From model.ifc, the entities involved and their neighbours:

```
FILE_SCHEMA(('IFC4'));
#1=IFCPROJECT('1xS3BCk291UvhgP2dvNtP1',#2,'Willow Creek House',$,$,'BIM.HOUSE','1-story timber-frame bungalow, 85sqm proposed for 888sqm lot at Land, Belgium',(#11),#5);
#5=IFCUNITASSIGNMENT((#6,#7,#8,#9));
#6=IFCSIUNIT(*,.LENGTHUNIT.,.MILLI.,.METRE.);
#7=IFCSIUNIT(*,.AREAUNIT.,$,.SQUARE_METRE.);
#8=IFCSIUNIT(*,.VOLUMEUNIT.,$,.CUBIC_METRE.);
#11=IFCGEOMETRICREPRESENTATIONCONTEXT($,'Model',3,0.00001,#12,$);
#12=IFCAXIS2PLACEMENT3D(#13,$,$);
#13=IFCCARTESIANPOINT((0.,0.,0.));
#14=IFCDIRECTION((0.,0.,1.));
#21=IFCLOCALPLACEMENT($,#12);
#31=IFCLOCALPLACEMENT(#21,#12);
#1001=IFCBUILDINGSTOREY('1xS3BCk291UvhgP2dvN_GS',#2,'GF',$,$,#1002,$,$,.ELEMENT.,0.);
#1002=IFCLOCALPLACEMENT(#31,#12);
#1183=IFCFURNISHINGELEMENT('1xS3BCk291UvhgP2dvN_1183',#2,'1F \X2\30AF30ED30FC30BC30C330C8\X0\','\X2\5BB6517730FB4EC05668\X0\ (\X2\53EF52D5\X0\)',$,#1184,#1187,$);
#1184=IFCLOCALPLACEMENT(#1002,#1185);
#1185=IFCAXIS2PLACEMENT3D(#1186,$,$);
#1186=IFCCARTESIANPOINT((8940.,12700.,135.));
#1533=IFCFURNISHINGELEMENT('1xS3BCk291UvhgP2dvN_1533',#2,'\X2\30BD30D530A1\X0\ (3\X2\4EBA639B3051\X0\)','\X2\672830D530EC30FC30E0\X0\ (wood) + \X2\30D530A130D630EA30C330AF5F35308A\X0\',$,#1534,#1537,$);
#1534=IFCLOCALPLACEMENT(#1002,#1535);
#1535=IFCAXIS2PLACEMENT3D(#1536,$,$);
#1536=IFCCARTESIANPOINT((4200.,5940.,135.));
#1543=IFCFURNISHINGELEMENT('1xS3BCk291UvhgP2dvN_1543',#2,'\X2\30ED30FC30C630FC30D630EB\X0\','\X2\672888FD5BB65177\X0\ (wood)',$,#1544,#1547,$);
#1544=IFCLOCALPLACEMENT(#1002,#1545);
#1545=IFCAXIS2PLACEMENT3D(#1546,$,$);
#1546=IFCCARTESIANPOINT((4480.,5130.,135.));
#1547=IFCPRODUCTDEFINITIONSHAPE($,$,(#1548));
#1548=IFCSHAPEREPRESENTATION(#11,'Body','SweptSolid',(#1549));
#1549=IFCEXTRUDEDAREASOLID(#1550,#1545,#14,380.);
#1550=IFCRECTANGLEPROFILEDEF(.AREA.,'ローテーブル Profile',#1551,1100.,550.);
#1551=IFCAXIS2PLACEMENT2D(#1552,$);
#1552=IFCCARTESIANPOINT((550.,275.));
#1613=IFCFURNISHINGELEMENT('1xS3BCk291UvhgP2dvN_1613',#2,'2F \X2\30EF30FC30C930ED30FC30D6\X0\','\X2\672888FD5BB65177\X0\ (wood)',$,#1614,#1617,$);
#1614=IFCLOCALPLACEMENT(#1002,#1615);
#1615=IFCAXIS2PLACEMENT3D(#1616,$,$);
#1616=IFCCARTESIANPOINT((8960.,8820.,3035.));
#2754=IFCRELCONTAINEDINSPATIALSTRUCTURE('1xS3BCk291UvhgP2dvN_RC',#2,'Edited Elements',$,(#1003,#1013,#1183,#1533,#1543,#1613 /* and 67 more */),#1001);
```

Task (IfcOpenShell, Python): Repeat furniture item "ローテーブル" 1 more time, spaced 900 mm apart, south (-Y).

```python
import numpy as np
import ifcopenshell
import ifcopenshell.api.geometry
import ifcopenshell.api.root
import ifcopenshell.util.element
import ifcopenshell.util.placement
import ifcopenshell.util.unit

model = ifcopenshell.open("model.ifc")
unit_scale = ifcopenshell.util.unit.calculate_unit_scale(model)


def reuse_history(source, copy):
    """copy_class also copies each property set's owner history, people and application; keep the originals."""
    for rel in copy.IsDefinedBy:
        if rel.is_a("IfcRelDefinesByProperties") and (history := rel.RelatingPropertyDefinition.OwnerHistory):
            rel.RelatingPropertyDefinition.OwnerHistory = source.OwnerHistory
            ifcopenshell.util.element.remove_deep2(model, history)


source = model.by_guid("1xS3BCk291UvhgP2dvN_1543")
base = ifcopenshell.util.placement.get_local_placement(source.ObjectPlacement)
step = np.array([0.0, -1.0, 0.0]) * 0.9 / unit_scale

for i in range(1, 2):
    copy = ifcopenshell.api.root.copy_class(model, product=source)
    copy.Representation = ifcopenshell.util.element.copy_deep(
        model, source.Representation, exclude=["IfcGeometricRepresentationContext", "IfcRepresentationMap"]
    )
    reuse_history(source, copy)
    matrix = base.copy()
    matrix[:3, 3] += i * step
    print("added at", matrix[:3, 3].round(3) + 0.0)
    ifcopenshell.api.geometry.edit_object_placement(model, product=copy, matrix=matrix, is_si=False)

model.write("model_updated.ifc")
```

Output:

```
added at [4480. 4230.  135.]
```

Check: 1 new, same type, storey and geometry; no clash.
